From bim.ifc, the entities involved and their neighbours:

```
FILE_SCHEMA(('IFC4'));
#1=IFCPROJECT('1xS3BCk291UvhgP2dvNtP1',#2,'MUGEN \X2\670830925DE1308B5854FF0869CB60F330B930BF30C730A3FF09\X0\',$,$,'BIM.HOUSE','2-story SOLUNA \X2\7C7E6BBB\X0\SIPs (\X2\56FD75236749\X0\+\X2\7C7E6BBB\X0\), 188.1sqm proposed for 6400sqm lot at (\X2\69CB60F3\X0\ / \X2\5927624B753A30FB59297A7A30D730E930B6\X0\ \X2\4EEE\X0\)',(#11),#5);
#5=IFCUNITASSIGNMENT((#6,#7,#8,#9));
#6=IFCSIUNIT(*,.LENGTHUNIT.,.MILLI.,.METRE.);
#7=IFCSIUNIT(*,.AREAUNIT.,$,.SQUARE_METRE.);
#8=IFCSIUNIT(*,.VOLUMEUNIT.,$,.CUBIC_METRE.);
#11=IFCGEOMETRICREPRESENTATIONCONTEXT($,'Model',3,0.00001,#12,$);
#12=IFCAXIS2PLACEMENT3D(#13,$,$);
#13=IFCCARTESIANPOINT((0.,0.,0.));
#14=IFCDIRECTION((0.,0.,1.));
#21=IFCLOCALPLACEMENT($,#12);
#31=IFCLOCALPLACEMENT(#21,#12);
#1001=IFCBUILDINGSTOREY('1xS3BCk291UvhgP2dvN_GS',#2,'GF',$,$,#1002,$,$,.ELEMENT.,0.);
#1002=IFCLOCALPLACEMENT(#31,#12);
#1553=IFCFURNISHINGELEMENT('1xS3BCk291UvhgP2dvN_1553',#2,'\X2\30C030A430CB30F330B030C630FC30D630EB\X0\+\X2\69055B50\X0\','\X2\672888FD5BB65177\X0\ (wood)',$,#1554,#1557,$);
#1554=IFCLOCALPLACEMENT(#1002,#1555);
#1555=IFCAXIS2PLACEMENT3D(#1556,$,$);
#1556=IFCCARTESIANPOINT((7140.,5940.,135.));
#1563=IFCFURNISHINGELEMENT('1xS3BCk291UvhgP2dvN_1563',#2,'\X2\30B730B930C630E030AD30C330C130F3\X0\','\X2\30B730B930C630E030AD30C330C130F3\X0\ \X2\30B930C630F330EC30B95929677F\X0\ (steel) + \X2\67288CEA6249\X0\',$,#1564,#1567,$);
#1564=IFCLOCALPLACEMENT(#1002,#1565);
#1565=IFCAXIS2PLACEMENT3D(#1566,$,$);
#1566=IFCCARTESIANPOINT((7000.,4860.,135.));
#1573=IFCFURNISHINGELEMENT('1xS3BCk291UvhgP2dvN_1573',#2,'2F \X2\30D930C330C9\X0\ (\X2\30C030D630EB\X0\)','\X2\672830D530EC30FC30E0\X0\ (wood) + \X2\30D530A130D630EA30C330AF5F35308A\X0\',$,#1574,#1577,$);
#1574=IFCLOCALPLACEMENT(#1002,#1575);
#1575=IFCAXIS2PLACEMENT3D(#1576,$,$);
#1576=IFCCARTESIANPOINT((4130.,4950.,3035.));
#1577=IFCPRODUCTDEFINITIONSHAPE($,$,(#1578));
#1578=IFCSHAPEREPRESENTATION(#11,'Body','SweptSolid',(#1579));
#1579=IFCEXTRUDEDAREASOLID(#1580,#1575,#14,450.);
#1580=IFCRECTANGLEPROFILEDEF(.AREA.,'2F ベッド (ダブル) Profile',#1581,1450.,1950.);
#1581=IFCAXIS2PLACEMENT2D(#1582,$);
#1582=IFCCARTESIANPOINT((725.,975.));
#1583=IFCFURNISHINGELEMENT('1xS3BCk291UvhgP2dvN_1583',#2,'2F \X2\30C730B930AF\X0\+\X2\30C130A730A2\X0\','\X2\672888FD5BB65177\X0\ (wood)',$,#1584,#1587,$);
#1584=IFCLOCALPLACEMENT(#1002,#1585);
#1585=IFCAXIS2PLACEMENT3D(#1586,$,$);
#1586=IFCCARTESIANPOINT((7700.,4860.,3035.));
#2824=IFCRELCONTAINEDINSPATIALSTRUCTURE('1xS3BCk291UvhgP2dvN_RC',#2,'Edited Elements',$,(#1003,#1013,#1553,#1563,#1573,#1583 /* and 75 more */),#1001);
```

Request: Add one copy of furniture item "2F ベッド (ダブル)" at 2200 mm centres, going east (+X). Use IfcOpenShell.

```python
import numpy as np
import ifcopenshell
import ifcopenshell.api.geometry
import ifcopenshell.api.root
import ifcopenshell.util.element
import ifcopenshell.util.placement
import ifcopenshell.util.unit

model = ifcopenshell.open("bim.ifc")
unit_scale = ifcopenshell.util.unit.calculate_unit_scale(model)


def reuse_history(source, copy):
    """copy_class also copies each property set's owner history, people and application; keep the originals."""
    for rel in copy.IsDefinedBy:
        if rel.is_a("IfcRelDefinesByProperties") and (history := rel.RelatingPropertyDefinition.OwnerHistory):
            rel.RelatingPropertyDefinition.OwnerHistory = source.OwnerHistory
            ifcopenshell.util.element.remove_deep2(model, history)


source = model.by_id(1573)
base = ifcopenshell.util.placement.get_local_placement(source.ObjectPlacement)
step = np.array([1.0, 0.0, 0.0]) * 2.2 / unit_scale

for i in range(1, 2):
    copy = ifcopenshell.api.root.copy_class(model, product=source)
    copy.Representation = ifcopenshell.util.element.copy_deep(
        model, source.Representation, exclude=["IfcGeometricRepresentationContext", "IfcRepresentationMap"]
    )
    reuse_history(source, copy)
    matrix = base.copy()
    matrix[:3, 3] += i * step
    print("added at", matrix[:3, 3].round(3) + 0.0)
    ifcopenshell.api.geometry.edit_object_placement(model, product=copy, matrix=matrix, is_si=False)

model.write("bim_edited.ifc")
```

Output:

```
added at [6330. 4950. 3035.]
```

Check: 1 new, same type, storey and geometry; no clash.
